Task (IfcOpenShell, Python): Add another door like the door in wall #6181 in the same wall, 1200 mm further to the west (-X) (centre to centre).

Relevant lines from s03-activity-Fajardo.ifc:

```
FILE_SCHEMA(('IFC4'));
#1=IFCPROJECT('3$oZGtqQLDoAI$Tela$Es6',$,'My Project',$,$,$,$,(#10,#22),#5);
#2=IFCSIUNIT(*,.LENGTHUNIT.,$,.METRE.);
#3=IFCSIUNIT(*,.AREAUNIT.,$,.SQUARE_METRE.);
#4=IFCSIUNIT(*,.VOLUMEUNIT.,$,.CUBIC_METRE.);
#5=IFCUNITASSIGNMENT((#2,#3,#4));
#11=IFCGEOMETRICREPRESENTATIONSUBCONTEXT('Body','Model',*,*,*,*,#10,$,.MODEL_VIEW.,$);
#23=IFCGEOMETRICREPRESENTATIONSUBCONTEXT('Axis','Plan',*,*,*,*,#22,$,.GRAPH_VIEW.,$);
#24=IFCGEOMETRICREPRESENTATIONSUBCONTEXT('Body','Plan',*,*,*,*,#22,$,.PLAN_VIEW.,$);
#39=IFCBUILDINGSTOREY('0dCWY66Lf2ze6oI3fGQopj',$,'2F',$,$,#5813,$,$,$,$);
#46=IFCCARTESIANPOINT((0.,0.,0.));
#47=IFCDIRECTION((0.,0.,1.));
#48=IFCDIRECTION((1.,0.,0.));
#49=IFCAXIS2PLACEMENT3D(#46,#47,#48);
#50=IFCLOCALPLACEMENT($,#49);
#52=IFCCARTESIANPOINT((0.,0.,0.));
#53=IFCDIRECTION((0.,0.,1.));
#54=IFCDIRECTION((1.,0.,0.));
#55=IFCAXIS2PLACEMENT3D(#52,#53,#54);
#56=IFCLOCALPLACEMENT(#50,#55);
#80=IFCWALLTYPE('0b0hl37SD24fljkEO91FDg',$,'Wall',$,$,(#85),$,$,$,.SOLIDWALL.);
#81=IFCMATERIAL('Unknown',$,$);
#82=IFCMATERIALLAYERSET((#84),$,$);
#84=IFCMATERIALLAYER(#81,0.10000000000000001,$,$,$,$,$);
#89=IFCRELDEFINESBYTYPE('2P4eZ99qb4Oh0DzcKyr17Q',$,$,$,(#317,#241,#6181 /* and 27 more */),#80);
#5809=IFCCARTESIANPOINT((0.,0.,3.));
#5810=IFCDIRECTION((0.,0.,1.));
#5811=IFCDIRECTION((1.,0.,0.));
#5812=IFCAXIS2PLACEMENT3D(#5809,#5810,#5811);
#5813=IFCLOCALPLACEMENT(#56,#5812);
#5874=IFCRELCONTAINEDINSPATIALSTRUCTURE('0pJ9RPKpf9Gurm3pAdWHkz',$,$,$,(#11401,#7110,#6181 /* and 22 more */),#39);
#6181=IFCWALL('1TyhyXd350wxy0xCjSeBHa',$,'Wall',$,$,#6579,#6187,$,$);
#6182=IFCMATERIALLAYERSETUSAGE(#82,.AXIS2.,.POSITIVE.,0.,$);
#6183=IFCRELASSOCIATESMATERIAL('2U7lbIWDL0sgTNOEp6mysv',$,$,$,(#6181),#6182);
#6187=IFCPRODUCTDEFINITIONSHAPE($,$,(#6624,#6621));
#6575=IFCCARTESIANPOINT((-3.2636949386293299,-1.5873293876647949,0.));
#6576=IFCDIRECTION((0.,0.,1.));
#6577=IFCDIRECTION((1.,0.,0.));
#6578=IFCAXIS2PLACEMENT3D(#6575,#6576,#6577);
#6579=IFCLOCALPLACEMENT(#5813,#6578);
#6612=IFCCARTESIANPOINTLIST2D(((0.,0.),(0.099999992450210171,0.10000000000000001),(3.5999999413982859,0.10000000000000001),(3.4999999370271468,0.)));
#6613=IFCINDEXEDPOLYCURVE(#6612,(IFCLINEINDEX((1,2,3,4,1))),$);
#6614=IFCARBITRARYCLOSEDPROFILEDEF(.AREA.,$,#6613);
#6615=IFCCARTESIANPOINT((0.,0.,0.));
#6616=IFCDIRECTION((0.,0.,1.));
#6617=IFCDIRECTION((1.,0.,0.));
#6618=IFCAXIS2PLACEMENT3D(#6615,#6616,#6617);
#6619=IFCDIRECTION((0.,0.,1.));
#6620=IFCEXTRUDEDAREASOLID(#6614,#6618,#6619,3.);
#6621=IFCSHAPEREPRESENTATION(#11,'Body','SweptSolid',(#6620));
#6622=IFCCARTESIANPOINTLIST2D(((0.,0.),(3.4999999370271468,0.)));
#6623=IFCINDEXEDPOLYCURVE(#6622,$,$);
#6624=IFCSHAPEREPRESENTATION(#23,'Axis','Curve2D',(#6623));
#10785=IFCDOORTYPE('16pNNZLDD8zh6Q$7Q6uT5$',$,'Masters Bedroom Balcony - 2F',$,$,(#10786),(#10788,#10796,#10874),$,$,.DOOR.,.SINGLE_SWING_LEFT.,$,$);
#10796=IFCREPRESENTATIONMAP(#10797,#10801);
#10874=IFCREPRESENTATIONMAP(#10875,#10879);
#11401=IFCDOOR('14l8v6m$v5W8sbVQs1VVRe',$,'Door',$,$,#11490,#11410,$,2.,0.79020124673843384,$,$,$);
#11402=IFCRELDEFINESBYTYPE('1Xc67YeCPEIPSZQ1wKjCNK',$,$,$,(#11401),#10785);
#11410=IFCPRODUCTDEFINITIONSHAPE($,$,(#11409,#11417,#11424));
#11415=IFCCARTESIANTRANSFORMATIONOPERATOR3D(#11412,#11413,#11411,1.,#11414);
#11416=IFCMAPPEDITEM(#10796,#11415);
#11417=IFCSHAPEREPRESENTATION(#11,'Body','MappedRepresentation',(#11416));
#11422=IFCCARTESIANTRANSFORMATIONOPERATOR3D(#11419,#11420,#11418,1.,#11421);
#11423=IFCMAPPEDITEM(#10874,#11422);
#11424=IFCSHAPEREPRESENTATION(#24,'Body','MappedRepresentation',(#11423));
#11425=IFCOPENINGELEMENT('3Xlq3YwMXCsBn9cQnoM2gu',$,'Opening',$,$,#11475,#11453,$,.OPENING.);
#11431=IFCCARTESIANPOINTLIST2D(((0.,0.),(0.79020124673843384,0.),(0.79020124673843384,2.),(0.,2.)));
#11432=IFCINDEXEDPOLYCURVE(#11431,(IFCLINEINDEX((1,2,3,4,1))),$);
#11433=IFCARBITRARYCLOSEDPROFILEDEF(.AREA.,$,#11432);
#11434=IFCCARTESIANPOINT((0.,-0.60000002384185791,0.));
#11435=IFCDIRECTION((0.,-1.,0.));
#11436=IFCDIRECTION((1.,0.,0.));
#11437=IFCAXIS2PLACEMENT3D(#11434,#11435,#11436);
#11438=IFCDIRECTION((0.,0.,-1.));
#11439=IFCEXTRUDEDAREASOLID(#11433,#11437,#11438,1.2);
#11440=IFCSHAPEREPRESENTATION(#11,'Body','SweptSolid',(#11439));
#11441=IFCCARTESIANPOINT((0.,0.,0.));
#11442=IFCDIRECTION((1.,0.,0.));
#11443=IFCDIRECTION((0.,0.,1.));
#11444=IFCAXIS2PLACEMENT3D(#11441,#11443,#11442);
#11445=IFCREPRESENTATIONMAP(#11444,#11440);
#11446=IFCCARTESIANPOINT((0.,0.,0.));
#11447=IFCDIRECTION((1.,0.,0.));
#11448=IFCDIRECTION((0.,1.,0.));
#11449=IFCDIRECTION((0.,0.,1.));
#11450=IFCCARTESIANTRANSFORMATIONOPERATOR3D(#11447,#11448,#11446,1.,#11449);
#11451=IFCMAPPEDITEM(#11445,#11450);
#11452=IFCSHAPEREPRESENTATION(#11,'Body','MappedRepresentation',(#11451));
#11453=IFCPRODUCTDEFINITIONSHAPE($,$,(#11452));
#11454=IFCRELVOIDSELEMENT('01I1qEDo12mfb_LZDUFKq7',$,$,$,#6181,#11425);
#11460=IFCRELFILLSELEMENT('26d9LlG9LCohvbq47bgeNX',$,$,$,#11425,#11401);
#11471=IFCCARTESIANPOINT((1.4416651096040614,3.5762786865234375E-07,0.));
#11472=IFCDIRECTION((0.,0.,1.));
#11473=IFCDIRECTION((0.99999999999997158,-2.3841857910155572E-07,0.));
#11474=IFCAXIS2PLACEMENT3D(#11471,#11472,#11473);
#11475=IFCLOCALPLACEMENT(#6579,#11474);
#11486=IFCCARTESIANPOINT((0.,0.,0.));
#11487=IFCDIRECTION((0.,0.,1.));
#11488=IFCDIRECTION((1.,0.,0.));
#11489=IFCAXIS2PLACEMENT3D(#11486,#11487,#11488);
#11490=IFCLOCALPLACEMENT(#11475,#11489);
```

```python
import ifcopenshell
import ifcopenshell.api.feature
import ifcopenshell.api.geometry
import ifcopenshell.api.root
import ifcopenshell.geom
import ifcopenshell.util.element
import ifcopenshell.util.placement
import ifcopenshell.util.shape
import ifcopenshell.util.unit

model = ifcopenshell.open("s03-activity-Fajardo.ifc")
unit_scale = ifcopenshell.util.unit.calculate_unit_scale(model)
settings = ifcopenshell.geom.settings()


def volume(element):
    """Net volume in cubic metres, openings subtracted."""
    shape = ifcopenshell.geom.create_shape(settings, element)
    return ifcopenshell.util.shape.get_volume(shape.geometry)


door = model.by_guid("14l8v6m$v5W8sbVQs1VVRe")
opening = door.FillsVoids[0].RelatingOpeningElement
wall = opening.VoidsElements[0].RelatingBuildingElement
before = volume(wall)
shift = ifcopenshell.util.placement.get_local_placement(wall.ObjectPlacement)[:3, 0] * -1.2 / unit_scale

# copy_class copies the void relationship, type, container and properties, but no geometry.
new_opening = ifcopenshell.api.root.copy_class(model, product=opening)
new_opening.Representation = ifcopenshell.util.element.copy_deep(
    model, opening.Representation, exclude=["IfcGeometricRepresentationContext", "IfcRepresentationMap"]
)
new_door = ifcopenshell.api.root.copy_class(model, product=door)
new_door.Representation = ifcopenshell.util.element.copy_deep(
    model, door.Representation, exclude=["IfcGeometricRepresentationContext", "IfcRepresentationMap"]
)
ifcopenshell.api.feature.add_filling(model, opening=new_opening, element=new_door)

for old, new in ((opening, new_opening), (door, new_door)):
    matrix = ifcopenshell.util.placement.get_local_placement(old.ObjectPlacement)
    matrix[:3, 3] += shift
    ifcopenshell.api.geometry.edit_object_placement(model, product=new, matrix=matrix, is_si=False)

after = volume(wall)

print(f"wall volume {before:.3f} -> {after:.3f} m3")

model.write("s03-activity-Fajardo-out.ifc")
```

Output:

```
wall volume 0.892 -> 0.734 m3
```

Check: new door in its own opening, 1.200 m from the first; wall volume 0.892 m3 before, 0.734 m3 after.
